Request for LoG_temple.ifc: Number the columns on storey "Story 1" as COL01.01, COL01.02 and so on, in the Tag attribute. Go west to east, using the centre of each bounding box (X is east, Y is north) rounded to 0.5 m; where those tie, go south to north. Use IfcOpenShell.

First a look at what the model holds.

```python
import ifcopenshell
import ifcopenshell.util.element
import ifcopenshell.util.placement

model = ifcopenshell.open("LoG_temple.ifc")
print(model.schema)
storey = next(s for s in model.by_type("IfcBuildingStorey") if s.Name == "Story 1")
columns = [e for e in ifcopenshell.util.element.get_decomposition(storey) if e.is_a("IfcColumn")]
for e in sorted(columns, key=lambda e: e.id()):
    origin = ifcopenshell.util.placement.get_local_placement(e.ObjectPlacement)[:3, 3]
    print(e.id(), e.Tag, e.Name, origin.round(2) + 0.0, sep=" | ")
```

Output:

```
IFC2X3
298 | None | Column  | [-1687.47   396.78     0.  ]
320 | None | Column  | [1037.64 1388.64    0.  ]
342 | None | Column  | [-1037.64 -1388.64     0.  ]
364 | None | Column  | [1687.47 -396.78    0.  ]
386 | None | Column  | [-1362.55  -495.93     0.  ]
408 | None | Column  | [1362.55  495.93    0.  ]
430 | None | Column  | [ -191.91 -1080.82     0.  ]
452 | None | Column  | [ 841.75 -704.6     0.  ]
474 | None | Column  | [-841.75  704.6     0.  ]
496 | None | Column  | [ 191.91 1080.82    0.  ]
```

```python
import ifcopenshell
import ifcopenshell.geom
import ifcopenshell.util.element
import ifcopenshell.util.shape

model = ifcopenshell.open("LoG_temple.ifc")
settings = ifcopenshell.geom.settings()
settings.set("use-world-coords", True)


def centre(element):
    shape = ifcopenshell.geom.create_shape(settings, element)
    return ifcopenshell.util.shape.get_bbox_centroid(shape.geometry)


storey = next(s for s in model.by_type("IfcBuildingStorey") if s.Name == "Story 1")
columns = [e for e in ifcopenshell.util.element.get_decomposition(storey) if e.is_a("IfcColumn")]

# Insertion points can sit at a corner or the storey origin, so sort by the geometry (in metres).
centres = {e: centre(e) for e in columns}
columns.sort(key=lambda e: (round(centres[e][0] / 0.5), centres[e][1]))

for i, e in enumerate(columns, start=1):
    number = f"COL01.{i:02d}"
    e.Tag = number
    print(e.id(), number)

model.write("LoG_temple_v2.ifc")
```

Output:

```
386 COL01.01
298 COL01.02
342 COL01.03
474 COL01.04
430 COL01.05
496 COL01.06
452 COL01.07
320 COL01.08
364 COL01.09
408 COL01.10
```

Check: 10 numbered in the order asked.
